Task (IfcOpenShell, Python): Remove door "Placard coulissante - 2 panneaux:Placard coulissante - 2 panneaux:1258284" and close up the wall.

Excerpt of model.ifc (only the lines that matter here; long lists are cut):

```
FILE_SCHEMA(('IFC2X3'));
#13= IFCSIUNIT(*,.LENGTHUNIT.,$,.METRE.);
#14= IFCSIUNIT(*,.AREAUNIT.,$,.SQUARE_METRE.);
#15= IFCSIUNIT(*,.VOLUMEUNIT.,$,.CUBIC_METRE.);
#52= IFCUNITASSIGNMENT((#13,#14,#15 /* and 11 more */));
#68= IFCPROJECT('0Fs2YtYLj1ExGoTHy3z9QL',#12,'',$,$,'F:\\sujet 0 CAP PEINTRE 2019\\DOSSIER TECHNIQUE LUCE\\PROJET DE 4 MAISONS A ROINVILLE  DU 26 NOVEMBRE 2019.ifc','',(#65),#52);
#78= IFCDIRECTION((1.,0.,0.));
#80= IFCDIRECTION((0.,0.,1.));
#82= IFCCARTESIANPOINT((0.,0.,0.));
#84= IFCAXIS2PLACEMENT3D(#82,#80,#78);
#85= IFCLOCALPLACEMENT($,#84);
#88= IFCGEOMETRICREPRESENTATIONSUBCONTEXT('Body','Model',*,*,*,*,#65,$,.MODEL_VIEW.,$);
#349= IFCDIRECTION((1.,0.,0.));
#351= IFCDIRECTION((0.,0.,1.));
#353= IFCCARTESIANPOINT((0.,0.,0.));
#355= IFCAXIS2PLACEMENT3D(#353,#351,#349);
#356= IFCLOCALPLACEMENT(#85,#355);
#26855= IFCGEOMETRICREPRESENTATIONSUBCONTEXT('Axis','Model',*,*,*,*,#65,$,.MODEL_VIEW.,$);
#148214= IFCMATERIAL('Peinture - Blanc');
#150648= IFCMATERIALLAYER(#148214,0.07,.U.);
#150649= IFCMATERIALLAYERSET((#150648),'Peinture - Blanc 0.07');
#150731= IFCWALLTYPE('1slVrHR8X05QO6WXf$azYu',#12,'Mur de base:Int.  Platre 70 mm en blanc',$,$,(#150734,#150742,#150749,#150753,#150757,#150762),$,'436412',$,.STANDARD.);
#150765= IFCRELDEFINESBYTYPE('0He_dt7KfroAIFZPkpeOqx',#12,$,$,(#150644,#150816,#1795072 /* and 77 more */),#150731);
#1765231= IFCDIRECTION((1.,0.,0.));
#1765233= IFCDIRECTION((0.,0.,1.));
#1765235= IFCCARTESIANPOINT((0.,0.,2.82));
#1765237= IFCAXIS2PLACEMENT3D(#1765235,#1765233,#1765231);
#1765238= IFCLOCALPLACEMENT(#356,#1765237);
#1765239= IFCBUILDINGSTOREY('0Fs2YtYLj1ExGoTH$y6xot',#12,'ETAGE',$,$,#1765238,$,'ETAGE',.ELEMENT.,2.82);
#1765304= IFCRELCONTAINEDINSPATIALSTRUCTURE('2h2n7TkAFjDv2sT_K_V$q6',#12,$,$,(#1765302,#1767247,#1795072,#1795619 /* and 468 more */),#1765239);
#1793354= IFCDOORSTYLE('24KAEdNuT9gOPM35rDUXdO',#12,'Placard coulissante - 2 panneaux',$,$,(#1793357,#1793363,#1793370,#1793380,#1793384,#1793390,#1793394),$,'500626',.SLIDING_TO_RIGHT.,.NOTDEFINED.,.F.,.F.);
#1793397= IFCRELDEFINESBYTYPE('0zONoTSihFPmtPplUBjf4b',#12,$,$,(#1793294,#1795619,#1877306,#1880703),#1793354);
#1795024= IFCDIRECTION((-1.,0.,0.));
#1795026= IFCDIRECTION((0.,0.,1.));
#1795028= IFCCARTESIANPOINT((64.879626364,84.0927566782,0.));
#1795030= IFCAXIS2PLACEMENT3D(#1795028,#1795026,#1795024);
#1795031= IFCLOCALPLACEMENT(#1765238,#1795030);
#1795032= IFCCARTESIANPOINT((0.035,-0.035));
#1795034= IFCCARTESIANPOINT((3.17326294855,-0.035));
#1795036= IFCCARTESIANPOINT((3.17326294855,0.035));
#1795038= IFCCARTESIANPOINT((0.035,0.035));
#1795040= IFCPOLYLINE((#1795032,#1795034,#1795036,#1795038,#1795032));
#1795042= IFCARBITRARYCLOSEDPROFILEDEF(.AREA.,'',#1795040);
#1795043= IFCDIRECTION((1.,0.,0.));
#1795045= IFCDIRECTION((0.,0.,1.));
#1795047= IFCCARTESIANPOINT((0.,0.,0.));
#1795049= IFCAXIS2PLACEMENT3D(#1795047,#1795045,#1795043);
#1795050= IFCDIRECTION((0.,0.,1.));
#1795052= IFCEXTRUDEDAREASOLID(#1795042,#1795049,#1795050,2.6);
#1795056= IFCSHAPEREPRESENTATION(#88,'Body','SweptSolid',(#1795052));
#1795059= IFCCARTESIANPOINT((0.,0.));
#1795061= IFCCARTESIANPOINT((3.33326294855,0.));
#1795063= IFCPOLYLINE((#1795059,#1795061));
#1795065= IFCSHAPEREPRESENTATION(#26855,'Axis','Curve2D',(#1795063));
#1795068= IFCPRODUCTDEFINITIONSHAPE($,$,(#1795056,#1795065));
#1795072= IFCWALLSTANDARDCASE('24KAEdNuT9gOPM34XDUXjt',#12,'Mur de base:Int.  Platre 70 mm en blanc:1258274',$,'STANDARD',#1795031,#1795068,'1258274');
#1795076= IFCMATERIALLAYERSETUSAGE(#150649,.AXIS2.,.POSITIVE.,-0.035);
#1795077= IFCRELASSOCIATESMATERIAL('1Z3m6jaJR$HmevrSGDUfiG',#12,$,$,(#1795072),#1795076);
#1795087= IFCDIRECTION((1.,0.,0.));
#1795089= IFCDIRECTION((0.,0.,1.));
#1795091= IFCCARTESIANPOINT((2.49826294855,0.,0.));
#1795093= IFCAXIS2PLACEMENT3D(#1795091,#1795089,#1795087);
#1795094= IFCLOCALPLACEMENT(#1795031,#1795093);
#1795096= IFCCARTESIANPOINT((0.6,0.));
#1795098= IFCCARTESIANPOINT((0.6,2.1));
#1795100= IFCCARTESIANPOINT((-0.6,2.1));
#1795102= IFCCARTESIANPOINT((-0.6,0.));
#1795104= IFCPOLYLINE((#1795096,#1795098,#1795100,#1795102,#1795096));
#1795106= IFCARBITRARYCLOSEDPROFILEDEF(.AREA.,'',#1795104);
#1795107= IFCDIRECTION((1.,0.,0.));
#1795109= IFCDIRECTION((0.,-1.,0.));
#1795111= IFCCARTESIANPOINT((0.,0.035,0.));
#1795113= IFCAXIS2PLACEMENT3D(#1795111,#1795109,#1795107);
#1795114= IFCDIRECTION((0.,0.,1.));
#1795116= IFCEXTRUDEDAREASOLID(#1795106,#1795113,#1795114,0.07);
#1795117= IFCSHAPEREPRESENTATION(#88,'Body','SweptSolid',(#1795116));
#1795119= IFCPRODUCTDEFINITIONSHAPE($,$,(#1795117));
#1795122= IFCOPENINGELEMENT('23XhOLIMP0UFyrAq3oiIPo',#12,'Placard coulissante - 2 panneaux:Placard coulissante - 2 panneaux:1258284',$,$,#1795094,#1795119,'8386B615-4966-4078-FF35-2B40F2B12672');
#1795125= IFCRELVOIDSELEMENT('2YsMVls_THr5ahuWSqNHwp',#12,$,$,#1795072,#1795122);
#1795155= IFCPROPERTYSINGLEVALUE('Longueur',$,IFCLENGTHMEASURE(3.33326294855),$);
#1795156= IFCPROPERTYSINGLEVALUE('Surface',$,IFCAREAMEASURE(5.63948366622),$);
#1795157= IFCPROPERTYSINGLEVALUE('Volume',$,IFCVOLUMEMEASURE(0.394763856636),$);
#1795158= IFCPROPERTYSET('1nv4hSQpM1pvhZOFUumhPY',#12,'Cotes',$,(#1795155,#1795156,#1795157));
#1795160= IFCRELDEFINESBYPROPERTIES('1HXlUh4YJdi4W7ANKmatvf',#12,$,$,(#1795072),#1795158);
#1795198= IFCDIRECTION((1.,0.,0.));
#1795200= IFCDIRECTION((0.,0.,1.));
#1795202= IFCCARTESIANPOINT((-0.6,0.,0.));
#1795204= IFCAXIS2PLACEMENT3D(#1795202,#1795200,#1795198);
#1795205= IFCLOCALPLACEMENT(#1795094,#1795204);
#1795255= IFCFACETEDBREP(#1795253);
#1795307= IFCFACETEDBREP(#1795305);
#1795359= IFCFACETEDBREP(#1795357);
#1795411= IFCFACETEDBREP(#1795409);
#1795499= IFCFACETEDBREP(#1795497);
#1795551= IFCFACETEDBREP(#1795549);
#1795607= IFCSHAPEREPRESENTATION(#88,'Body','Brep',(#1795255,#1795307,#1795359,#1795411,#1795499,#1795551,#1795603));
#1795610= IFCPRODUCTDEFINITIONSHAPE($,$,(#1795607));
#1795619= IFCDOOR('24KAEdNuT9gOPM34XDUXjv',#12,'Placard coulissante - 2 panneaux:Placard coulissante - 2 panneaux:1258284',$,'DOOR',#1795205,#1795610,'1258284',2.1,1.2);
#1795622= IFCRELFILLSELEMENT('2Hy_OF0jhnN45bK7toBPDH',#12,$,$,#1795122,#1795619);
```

```python
import ifcopenshell
import ifcopenshell.api.feature
import ifcopenshell.api.pset
import ifcopenshell.api.root
import ifcopenshell.geom
import ifcopenshell.util.element
import ifcopenshell.util.shape
import ifcopenshell.util.unit

model = ifcopenshell.open("model.ifc")
area_scale = ifcopenshell.util.unit.calculate_unit_scale(model, "AREAUNIT")
volume_scale = ifcopenshell.util.unit.calculate_unit_scale(model, "VOLUMEUNIT")
settings = ifcopenshell.geom.settings()


def volume(element):
    """Net volume in cubic metres, openings subtracted."""
    shape = ifcopenshell.geom.create_shape(settings, element)
    return ifcopenshell.util.shape.get_volume(shape.geometry)


door = model.by_guid("24KAEdNuT9gOPM34XDUXjv")
opening = door.FillsVoids[0].RelatingOpeningElement
wall = opening.VoidsElements[0].RelatingBuildingElement
before = volume(wall)

ifcopenshell.api.root.remove_product(model, product=door)
ifcopenshell.api.feature.remove_feature(model, feature=opening)

after = volume(wall)
thickness = 0.07  # wall thickness in metres

# Update the wall's stored quantities.
pset = model.by_id(ifcopenshell.util.element.get_pset(wall, "Cotes", should_inherit=False)["id"])
ifcopenshell.api.pset.edit_pset(model, pset=pset, properties={
    "Surface": model.create_entity("IfcAreaMeasure", after / thickness / area_scale),
    "Volume": model.create_entity("IfcVolumeMeasure", after / volume_scale),
})

print(f"wall volume {before:.3f} -> {after:.3f} m3")

model.write("model_v2.ifc")
```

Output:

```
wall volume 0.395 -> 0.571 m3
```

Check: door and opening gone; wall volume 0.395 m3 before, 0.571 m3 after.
